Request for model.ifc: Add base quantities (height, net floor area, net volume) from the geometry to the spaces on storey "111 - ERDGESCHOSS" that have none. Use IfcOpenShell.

First a look at what the model holds.

```python
import ifcopenshell
import ifcopenshell.util.element
import ifcopenshell.util.unit

model = ifcopenshell.open("model.ifc")
print(model.schema)
for unit_type in ("LENGTHUNIT", "AREAUNIT", "VOLUMEUNIT"):
    print(unit_type, ifcopenshell.util.unit.calculate_unit_scale(model, unit_type))
storey = next(s for s in model.by_type("IfcBuildingStorey") if s.Name == "111 - ERDGESCHOSS")
spaces = [e for e in ifcopenshell.util.element.get_decomposition(storey) if e.is_a("IfcSpace")]
for e in sorted(spaces, key=lambda e: e.id()):
    print(e.id(), e.is_a(), e.Name, list(ifcopenshell.util.element.get_psets(e, qtos_only=True)), sep=" | ")
```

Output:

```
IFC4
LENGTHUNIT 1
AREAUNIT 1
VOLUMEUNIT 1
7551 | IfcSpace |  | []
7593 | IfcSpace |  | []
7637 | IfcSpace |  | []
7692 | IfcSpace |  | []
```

```python
import ifcopenshell
import ifcopenshell.api.pset
import ifcopenshell.geom
import ifcopenshell.util.element
import ifcopenshell.util.shape
import ifcopenshell.util.unit

model = ifcopenshell.open("model.ifc")
unit_scale = ifcopenshell.util.unit.calculate_unit_scale(model)
area_scale = ifcopenshell.util.unit.calculate_unit_scale(model, "AREAUNIT")
volume_scale = ifcopenshell.util.unit.calculate_unit_scale(model, "VOLUMEUNIT")
settings = ifcopenshell.geom.settings()

storey = next(s for s in model.by_type("IfcBuildingStorey") if s.Name == "111 - ERDGESCHOSS")
spaces = [e for e in ifcopenshell.util.element.get_decomposition(storey) if e.is_a("IfcSpace")]

for e in sorted(spaces, key=lambda e: e.id()):
    if ifcopenshell.util.element.get_psets(e, qtos_only=True, should_inherit=False):
        continue
    # Geometry comes back in metres, in the element's own axes.
    shape = ifcopenshell.geom.create_shape(settings, e)
    values = {
        "Height": ifcopenshell.util.shape.get_z(shape.geometry) / unit_scale,
        "NetFloorArea": ifcopenshell.util.shape.get_footprint_area(shape.geometry) / area_scale,
        "NetVolume": ifcopenshell.util.shape.get_volume(shape.geometry) / volume_scale,
    }
    qto = ifcopenshell.api.pset.add_qto(model, product=e, name="Qto_SpaceBaseQuantities")
    ifcopenshell.api.pset.edit_qto(model, qto=qto, properties=values)
    print(e.id(), {k: round(v, 3) for k, v in values.items()})

model.write("model-out.ifc")
```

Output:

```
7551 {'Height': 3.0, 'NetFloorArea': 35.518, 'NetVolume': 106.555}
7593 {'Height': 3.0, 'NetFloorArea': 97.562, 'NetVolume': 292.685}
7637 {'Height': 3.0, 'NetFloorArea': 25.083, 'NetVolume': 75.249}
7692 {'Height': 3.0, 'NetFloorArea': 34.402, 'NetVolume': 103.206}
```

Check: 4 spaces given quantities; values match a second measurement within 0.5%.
